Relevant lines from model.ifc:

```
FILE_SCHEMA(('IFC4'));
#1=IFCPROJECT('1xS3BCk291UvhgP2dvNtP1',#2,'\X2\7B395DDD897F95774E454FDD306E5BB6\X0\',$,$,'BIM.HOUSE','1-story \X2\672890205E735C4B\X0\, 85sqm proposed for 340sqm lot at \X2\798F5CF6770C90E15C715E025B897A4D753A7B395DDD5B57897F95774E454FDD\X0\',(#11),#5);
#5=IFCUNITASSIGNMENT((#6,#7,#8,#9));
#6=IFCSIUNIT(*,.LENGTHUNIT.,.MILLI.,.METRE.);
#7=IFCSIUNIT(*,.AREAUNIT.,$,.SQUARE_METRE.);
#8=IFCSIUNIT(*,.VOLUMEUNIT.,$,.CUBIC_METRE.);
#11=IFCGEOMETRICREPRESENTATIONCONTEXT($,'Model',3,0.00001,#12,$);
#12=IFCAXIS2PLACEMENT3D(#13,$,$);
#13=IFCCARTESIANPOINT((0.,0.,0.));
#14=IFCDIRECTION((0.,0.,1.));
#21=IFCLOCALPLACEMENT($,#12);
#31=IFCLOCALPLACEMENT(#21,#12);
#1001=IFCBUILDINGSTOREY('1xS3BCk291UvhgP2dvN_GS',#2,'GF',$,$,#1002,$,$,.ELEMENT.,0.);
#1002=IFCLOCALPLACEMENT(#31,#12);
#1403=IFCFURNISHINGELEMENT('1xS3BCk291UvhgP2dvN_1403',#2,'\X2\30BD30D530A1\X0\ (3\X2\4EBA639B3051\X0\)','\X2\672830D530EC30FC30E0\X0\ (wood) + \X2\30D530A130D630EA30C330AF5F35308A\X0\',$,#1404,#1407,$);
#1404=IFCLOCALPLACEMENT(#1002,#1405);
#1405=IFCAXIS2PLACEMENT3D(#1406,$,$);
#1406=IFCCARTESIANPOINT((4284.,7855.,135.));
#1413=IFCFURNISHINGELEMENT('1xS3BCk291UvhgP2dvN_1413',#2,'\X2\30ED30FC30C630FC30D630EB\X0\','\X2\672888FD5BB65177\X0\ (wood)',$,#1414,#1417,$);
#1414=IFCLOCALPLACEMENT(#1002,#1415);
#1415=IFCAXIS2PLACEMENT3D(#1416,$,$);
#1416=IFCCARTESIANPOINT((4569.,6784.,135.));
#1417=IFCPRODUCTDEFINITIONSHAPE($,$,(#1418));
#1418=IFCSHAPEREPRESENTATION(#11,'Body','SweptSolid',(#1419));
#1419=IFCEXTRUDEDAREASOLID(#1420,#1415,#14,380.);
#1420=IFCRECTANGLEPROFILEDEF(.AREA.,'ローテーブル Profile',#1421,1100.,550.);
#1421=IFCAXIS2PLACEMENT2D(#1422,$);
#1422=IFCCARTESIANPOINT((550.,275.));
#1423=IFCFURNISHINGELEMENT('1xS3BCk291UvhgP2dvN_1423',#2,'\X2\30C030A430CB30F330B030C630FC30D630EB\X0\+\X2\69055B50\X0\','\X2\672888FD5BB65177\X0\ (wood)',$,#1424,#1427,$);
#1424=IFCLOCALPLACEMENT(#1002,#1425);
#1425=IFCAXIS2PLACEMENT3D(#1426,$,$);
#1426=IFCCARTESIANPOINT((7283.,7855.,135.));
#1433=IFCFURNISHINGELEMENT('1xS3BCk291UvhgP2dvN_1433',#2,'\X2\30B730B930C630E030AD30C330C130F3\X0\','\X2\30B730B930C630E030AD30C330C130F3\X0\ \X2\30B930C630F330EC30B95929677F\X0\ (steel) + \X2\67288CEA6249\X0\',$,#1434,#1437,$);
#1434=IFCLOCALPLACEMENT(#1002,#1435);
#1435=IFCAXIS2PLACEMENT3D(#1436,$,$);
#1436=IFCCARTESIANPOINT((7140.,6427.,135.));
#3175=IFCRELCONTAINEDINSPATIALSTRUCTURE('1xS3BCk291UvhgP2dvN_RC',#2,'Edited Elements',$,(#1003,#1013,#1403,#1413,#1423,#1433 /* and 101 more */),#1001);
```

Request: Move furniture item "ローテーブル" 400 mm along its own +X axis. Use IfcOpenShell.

```python
import ifcopenshell
import ifcopenshell.api.geometry
import ifcopenshell.util.placement
import ifcopenshell.util.unit

model = ifcopenshell.open("model.ifc")
unit_scale = ifcopenshell.util.unit.calculate_unit_scale(model)

item = model.by_guid("1xS3BCk291UvhgP2dvN_1413")
matrix = ifcopenshell.util.placement.get_local_placement(item.ObjectPlacement)
matrix[:3, 3] += matrix[:3, 0] * 0.4 / unit_scale
ifcopenshell.api.geometry.edit_object_placement(model, product=item, matrix=matrix, is_si=False)

print(ifcopenshell.util.placement.get_local_placement(item.ObjectPlacement).round(3) + 0.0)

model.write("model_updated.ifc")
```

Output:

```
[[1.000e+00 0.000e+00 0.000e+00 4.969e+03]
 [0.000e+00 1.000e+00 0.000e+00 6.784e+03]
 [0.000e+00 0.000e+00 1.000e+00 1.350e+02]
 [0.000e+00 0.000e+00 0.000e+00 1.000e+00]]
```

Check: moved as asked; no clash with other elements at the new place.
